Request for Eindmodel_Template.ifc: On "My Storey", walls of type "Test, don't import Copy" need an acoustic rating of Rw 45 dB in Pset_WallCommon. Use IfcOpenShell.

First a look at what the model holds.

```python
import ifcopenshell
import ifcopenshell.util.element

model = ifcopenshell.open("Eindmodel_Template.ifc")
print(model.schema)
storey = next(s for s in model.by_type("IfcBuildingStorey") if s.Name == "My Storey")
walls = [e for e in ifcopenshell.util.element.get_decomposition(storey) if e.is_a("IfcWall")]
seen = {}
for e in walls:
    element_type = ifcopenshell.util.element.get_type(e)
    key = (element_type.Name if element_type != e and element_type else None, ifcopenshell.util.element.get_pset(e, "Pset_WallCommon", "AcousticRating"))
    seen[key] = seen.get(key, 0) + 1
for (name, value), count in sorted(seen.items(), key=str):
    print(count, "x", name, "|", value)
```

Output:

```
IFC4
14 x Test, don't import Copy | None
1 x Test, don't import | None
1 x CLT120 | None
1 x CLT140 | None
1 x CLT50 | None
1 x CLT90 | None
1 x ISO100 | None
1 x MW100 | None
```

```python
import ifcopenshell
import ifcopenshell.api.pset
import ifcopenshell.util.element

model = ifcopenshell.open("Eindmodel_Template.ifc")

storey = next(s for s in model.by_type("IfcBuildingStorey") if s.Name == "My Storey")
walls = [e for e in ifcopenshell.util.element.get_decomposition(storey) if e.is_a("IfcWall")]

count = 0
for e in walls:
    element_type = ifcopenshell.util.element.get_type(e)
    if element_type in (None, e) or element_type.Name != "Test, don't import Copy":
        continue
    # add_pset returns the element's existing set when there is one.
    pset = ifcopenshell.api.pset.add_pset(model, product=e, name="Pset_WallCommon")
    ifcopenshell.api.pset.edit_pset(model, pset=pset, properties={"AcousticRating": "Rw 45 dB"})
    count += 1

print(count, "walls updated")

model.write("Eindmodel_Template_updated.ifc")
```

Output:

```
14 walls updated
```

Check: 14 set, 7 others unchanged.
